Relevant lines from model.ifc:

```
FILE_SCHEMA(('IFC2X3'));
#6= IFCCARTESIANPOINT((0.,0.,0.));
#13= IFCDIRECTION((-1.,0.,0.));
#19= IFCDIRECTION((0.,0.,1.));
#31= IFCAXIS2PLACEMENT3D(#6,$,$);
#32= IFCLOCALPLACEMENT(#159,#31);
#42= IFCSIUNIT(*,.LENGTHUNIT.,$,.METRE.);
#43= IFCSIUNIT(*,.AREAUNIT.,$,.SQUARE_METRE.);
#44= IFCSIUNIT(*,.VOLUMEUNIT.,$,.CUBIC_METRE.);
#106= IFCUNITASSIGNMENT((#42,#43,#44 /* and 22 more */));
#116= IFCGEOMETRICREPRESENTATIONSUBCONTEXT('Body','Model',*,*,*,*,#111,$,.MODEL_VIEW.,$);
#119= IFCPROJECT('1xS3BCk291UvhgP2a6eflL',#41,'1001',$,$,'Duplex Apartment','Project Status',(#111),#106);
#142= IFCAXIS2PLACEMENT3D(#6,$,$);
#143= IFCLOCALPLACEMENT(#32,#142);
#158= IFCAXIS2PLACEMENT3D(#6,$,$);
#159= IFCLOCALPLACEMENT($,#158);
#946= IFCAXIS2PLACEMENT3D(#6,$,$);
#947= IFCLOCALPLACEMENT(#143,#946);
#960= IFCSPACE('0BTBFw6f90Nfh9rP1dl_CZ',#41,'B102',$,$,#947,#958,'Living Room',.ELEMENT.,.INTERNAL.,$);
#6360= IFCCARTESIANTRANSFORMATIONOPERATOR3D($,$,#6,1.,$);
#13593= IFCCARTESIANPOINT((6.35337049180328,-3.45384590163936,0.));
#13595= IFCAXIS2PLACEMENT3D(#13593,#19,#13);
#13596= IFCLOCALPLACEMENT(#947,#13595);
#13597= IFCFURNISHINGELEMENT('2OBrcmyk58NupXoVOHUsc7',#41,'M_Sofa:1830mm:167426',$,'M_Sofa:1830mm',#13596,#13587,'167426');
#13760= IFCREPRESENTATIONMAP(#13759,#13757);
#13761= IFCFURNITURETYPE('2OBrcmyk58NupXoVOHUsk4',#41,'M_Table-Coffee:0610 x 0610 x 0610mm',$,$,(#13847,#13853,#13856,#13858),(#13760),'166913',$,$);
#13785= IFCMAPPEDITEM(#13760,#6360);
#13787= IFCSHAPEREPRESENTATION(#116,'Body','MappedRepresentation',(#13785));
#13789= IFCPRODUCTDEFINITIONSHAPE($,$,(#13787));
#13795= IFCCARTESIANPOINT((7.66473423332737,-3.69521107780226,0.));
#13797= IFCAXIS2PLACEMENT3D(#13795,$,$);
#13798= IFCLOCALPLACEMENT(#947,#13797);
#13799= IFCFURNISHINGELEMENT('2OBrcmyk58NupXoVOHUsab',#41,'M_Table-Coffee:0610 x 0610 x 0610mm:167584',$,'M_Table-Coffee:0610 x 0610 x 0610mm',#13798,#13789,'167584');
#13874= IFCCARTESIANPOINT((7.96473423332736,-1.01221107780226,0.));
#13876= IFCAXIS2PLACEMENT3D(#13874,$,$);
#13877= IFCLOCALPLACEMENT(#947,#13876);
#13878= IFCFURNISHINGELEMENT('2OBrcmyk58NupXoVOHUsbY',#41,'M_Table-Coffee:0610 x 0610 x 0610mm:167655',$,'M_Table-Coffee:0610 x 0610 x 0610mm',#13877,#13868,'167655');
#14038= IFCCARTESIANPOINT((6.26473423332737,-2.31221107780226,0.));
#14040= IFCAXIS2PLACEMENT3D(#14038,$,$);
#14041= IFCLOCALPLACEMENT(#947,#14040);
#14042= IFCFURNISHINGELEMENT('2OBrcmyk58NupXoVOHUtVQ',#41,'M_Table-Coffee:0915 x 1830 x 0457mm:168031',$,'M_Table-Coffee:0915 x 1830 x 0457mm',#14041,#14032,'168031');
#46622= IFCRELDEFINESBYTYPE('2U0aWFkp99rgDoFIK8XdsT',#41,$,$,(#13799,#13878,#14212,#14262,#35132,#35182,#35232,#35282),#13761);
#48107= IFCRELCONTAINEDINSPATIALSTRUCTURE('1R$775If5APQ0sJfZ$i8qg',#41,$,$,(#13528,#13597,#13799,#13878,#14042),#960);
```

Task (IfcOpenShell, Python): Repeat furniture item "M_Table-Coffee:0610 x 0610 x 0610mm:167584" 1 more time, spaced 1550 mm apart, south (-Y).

```python
import numpy as np
import ifcopenshell
import ifcopenshell.api.geometry
import ifcopenshell.api.root
import ifcopenshell.util.element
import ifcopenshell.util.placement

model = ifcopenshell.open("model.ifc")


def reuse_history(source, copy):
    """copy_class also copies each property set's owner history, people and application; keep the originals."""
    for rel in copy.IsDefinedBy:
        if rel.is_a("IfcRelDefinesByProperties") and (history := rel.RelatingPropertyDefinition.OwnerHistory):
            rel.RelatingPropertyDefinition.OwnerHistory = source.OwnerHistory
            ifcopenshell.util.element.remove_deep2(model, history)


source = model.by_guid("2OBrcmyk58NupXoVOHUsab")
base = ifcopenshell.util.placement.get_local_placement(source.ObjectPlacement)
step = np.array([0.0, -1.0, 0.0]) * 1.55

for i in range(1, 2):
    copy = ifcopenshell.api.root.copy_class(model, product=source)
    copy.Representation = ifcopenshell.util.element.copy_deep(
        model, source.Representation, exclude=["IfcGeometricRepresentationContext", "IfcRepresentationMap"]
    )
    copy.Name = "M_Table-Coffee:0610 x 0610 x 0610mm"
    copy.Tag = None
    reuse_history(source, copy)
    matrix = base.copy()
    matrix[:3, 3] += i * step
    print("added at", matrix[:3, 3].round(3) + 0.0)
    ifcopenshell.api.geometry.edit_object_placement(model, product=copy, matrix=matrix, is_si=False)

model.write("model_v2.ifc")
```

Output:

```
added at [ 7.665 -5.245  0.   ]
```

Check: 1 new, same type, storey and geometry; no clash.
